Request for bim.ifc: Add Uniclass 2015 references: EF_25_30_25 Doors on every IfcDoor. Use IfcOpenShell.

First a look at what the model holds.

```python
import ifcopenshell

model = ifcopenshell.open("bim.ifc")
print(model.schema)
print("classifications:", [c.Name for c in model.by_type("IfcClassification")])
for ifc_class in ("IfcDoor", "IfcRoof", "IfcStair", "IfcWall", "IfcWindow"):
    print(ifc_class, len(model.by_type(ifc_class)))
```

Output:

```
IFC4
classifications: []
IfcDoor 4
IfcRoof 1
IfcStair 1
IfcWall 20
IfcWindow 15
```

```python
import ifcopenshell
import ifcopenshell.api.classification

model = ifcopenshell.open("bim.ifc")

system = ifcopenshell.api.classification.add_classification(model, classification="Uniclass 2015")

codes = {
    "IfcDoor": ("EF_25_30_25", "Doors"),
}
for ifc_class, (code, name) in codes.items():
    products = model.by_type(ifc_class)
    ifcopenshell.api.classification.add_reference(
        model, products=products, classification=system, identification=code, name=name
    )
    print(code, len(products))

model.write("bim_edited.ifc")
```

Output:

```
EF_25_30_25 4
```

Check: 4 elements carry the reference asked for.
